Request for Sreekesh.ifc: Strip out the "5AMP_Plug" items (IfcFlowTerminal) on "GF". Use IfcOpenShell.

First a look at what the model holds.

```python
import ifcopenshell
import ifcopenshell.util.element

model = ifcopenshell.open("Sreekesh.ifc")
print(model.schema)
storey = next(s for s in model.by_type("IfcBuildingStorey") if s.Name == "GF")
terminals = [e for e in ifcopenshell.util.element.get_decomposition(storey) if e.is_a("IfcFlowTerminal")]
seen = {}
for e in terminals:
    element_type = ifcopenshell.util.element.get_type(e)
    name = element_type.Name if element_type not in (None, e) else None
    seen[name] = seen.get(name, 0) + 1
for name, count in sorted(seen.items(), key=str):
    print(count, "x", name)
```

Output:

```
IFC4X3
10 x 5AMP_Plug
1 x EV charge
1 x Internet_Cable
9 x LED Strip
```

```python
import ifcopenshell
import ifcopenshell.api.root
import ifcopenshell.util.element

model = ifcopenshell.open("Sreekesh.ifc")

storey = next(s for s in model.by_type("IfcBuildingStorey") if s.Name == "GF")
terminals = [e for e in ifcopenshell.util.element.get_decomposition(storey) if e.is_a("IfcFlowTerminal")]
targets = [e for e in terminals if (t := ifcopenshell.util.element.get_type(e)) not in (None, e) and t.Name == "5AMP_Plug"]

for e in targets:
    ifcopenshell.api.root.remove_product(model, product=e)
print(len(targets), "removed")

model.write("Sreekesh_updated.ifc")
```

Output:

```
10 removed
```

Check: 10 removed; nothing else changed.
